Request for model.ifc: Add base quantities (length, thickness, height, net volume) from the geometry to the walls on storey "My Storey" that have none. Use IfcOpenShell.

First a look at what the model holds.

```python
import ifcopenshell
import ifcopenshell.util.element
import ifcopenshell.util.unit

model = ifcopenshell.open("model.ifc")
print(model.schema)
for unit_type in ("LENGTHUNIT", "AREAUNIT", "VOLUMEUNIT"):
    print(unit_type, ifcopenshell.util.unit.calculate_unit_scale(model, unit_type))
storey = next(s for s in model.by_type("IfcBuildingStorey") if s.Name == "My Storey")
walls = [e for e in ifcopenshell.util.element.get_decomposition(storey) if e.is_a("IfcWall")]
for e in sorted(walls, key=lambda e: e.id()):
    print(e.id(), e.is_a(), e.Name, list(ifcopenshell.util.element.get_psets(e, qtos_only=True)), sep=" | ")
```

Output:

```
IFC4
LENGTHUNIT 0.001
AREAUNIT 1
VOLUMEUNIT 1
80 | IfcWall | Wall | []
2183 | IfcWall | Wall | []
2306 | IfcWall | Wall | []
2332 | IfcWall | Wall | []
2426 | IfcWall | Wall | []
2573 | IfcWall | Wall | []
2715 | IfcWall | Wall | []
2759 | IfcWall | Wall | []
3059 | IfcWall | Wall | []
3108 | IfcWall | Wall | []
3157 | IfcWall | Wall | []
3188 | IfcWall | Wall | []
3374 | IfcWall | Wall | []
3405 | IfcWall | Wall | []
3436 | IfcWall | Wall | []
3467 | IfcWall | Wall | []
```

```python
import ifcopenshell
import ifcopenshell.api.pset
import ifcopenshell.geom
import ifcopenshell.util.element
import ifcopenshell.util.shape
import ifcopenshell.util.unit

model = ifcopenshell.open("model.ifc")
unit_scale = ifcopenshell.util.unit.calculate_unit_scale(model)
volume_scale = ifcopenshell.util.unit.calculate_unit_scale(model, "VOLUMEUNIT")
settings = ifcopenshell.geom.settings()

storey = next(s for s in model.by_type("IfcBuildingStorey") if s.Name == "My Storey")
walls = [e for e in ifcopenshell.util.element.get_decomposition(storey) if e.is_a("IfcWall")]

for e in sorted(walls, key=lambda e: e.id()):
    if ifcopenshell.util.element.get_psets(e, qtos_only=True, should_inherit=False):
        continue
    # Geometry comes back in metres, in the element's own axes.
    shape = ifcopenshell.geom.create_shape(settings, e)
    values = {
        "Length": ifcopenshell.util.shape.get_x(shape.geometry) / unit_scale,
        "Width": ifcopenshell.util.shape.get_y(shape.geometry) / unit_scale,
        "Height": ifcopenshell.util.shape.get_z(shape.geometry) / unit_scale,
        "NetVolume": ifcopenshell.util.shape.get_volume(shape.geometry) / volume_scale,
    }
    qto = ifcopenshell.api.pset.add_qto(model, product=e, name="Qto_WallBaseQuantities")
    ifcopenshell.api.pset.edit_qto(model, qto=qto, properties=values)
    print(e.id(), {k: round(v, 3) for k, v in values.items()})

model.write("model_v2.ifc")
```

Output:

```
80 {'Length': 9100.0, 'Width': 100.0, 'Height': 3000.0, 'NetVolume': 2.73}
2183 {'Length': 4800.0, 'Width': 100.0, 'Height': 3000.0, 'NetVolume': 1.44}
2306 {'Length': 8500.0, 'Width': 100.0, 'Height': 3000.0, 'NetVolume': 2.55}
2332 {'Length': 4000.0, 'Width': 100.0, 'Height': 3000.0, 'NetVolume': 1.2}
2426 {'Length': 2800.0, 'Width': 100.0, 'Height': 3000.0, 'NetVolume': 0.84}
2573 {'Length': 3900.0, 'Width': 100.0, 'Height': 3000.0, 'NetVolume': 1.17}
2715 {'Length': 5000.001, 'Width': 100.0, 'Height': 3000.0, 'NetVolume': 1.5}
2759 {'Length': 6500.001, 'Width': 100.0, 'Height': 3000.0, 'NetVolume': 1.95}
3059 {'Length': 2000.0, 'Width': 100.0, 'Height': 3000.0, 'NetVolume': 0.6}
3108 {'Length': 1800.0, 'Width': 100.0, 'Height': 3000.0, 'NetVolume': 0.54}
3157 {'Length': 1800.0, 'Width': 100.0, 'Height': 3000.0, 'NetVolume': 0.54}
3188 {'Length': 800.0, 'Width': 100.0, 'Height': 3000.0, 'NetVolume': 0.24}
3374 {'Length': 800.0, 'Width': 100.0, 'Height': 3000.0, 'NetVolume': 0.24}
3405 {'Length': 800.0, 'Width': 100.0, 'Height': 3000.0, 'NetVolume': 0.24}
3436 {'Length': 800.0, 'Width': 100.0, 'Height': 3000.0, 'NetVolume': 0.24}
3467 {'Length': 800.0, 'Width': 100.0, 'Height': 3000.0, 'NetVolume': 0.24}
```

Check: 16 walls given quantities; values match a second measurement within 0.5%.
